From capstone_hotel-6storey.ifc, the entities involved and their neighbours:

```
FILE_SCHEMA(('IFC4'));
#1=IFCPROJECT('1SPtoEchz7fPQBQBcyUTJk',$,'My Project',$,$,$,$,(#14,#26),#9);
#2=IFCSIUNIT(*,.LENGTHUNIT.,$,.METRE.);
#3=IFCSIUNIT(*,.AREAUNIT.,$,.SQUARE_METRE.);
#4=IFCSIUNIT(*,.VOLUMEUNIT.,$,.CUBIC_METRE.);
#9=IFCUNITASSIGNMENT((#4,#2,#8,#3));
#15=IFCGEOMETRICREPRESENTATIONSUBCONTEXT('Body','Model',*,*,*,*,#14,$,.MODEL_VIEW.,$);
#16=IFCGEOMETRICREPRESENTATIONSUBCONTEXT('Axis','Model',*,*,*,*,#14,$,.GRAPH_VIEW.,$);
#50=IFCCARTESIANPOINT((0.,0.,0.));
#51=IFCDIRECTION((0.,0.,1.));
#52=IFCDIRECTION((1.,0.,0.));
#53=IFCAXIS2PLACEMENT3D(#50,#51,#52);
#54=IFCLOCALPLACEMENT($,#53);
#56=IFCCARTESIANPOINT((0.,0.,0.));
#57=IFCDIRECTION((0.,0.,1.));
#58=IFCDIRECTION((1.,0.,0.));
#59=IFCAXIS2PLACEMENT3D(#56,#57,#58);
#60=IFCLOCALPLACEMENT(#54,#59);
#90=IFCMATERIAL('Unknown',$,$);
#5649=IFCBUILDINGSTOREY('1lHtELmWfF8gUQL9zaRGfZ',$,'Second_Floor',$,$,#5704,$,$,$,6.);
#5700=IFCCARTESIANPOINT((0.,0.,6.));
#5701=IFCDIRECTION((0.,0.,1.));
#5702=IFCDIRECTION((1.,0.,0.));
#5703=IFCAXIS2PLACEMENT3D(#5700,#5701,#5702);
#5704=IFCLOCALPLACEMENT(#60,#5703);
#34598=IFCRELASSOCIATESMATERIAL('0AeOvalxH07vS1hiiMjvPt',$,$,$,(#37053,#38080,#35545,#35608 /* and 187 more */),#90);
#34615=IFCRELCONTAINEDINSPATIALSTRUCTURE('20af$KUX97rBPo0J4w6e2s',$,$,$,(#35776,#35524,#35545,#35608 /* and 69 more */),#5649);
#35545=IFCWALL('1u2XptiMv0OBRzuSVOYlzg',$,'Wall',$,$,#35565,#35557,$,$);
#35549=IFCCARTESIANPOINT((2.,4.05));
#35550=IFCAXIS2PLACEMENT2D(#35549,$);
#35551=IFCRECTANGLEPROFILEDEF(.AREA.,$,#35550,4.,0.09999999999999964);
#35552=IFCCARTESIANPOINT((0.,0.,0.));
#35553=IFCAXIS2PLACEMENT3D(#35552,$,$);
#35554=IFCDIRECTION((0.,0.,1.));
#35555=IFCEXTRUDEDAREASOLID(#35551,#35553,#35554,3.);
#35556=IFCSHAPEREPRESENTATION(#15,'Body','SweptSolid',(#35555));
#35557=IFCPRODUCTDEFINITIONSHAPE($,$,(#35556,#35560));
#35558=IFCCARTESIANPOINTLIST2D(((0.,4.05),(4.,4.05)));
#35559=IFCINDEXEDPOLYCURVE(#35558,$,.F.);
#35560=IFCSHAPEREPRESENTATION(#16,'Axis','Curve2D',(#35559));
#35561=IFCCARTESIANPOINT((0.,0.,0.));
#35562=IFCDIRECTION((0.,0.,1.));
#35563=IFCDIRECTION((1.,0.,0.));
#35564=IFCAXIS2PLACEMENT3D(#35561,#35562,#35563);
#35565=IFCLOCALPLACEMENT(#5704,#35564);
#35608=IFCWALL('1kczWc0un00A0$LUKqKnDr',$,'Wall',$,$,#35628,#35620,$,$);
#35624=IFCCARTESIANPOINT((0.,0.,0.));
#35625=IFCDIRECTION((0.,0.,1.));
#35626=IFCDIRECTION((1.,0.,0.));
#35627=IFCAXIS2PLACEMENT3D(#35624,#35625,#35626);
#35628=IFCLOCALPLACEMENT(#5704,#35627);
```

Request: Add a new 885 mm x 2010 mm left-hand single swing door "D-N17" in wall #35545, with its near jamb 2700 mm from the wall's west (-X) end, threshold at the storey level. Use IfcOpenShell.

```python
import numpy as np
import ifcopenshell
import ifcopenshell.api.feature
import ifcopenshell.api.geometry
import ifcopenshell.api.root
import ifcopenshell.api.spatial
import ifcopenshell.geom
import ifcopenshell.util.element
import ifcopenshell.util.placement
import ifcopenshell.util.representation
import ifcopenshell.util.shape
import ifcopenshell.util.unit

model = ifcopenshell.open("capstone_hotel-6storey.ifc")
unit_scale = ifcopenshell.util.unit.calculate_unit_scale(model)
settings = ifcopenshell.geom.settings()


def volume(element):
    """Net volume in cubic metres, openings subtracted."""
    shape = ifcopenshell.geom.create_shape(settings, element)
    return ifcopenshell.util.shape.get_volume(shape.geometry)


wall = model.by_guid("1u2XptiMv0OBRzuSVOYlzg")
storey = ifcopenshell.util.element.get_container(wall, ifc_class="IfcBuildingStorey")
context = ifcopenshell.util.representation.get_context(model, "Model", "Body", "MODEL_VIEW")
before = volume(wall)

width, height, from_end, sill = 0.885, 2.01, 2.7, 0.0  # metres

# The wall runs along its own X axis, and the end named is its -X end.
wall_shape = ifcopenshell.geom.create_shape(settings, wall)
x, y, z = ifcopenshell.util.shape.get_vertices(wall_shape.geometry).T
start = x.min() + from_end
face, thickness = float(y.min()), float(y.max() - y.min())
wall_matrix = ifcopenshell.util.placement.get_local_placement(wall.ObjectPlacement)
level = ifcopenshell.util.placement.get_local_placement(storey.ObjectPlacement)[2, 3]


def in_wall(x, y):
    """Placement at x, y metres in the wall's axes, at sill height."""
    matrix = wall_matrix.copy()
    matrix[:, 3] = wall_matrix @ np.array([x / unit_scale, y / unit_scale, 0.0, 1.0])
    matrix[2, 3] = level + sill / unit_scale
    return matrix


# Opening: a box that overshoots both wall faces by 50 mm.
opening = ifcopenshell.api.root.create_entity(model, ifc_class="IfcOpeningElement", predefined_type="OPENING")
box = ifcopenshell.api.geometry.add_wall_representation(
    model, context=context, length=width, height=height, thickness=thickness + 0.1
)
ifcopenshell.api.geometry.assign_representation(model, product=opening, representation=box)
ifcopenshell.api.geometry.edit_object_placement(model, product=opening, matrix=in_wall(start, face - 0.05), is_si=False)
ifcopenshell.api.feature.add_feature(model, feature=opening, element=wall)

door = ifcopenshell.api.root.create_entity(model, ifc_class="IfcDoor", name="D-N17", predefined_type="DOOR")
door.OverallWidth, door.OverallHeight = width / unit_scale, height / unit_scale
door.OperationType = "SINGLE_SWING_LEFT"
body = ifcopenshell.api.geometry.add_door_representation(
    model,
    context=context,
    overall_width=door.OverallWidth,
    overall_height=door.OverallHeight,
    operation_type="SINGLE_SWING_LEFT",
    lining_properties={"LiningDepth": thickness / unit_scale, "ThresholdDepth": thickness / unit_scale},
)
ifcopenshell.api.geometry.assign_representation(model, product=door, representation=body)
ifcopenshell.api.spatial.assign_container(model, products=[door], relating_structure=storey)
ifcopenshell.api.feature.add_filling(model, opening=opening, element=door)

# The lining spans the wall, so the door starts at the wall face.
ifcopenshell.api.geometry.edit_object_placement(model, product=door, matrix=in_wall(start, face), is_si=False)

after = volume(wall)

print(f"wall volume {before:.3f} -> {after:.3f} m3")

model.write("capstone_hotel-6storey_v2.ifc")
```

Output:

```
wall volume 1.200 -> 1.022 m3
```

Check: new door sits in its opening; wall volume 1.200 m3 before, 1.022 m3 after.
